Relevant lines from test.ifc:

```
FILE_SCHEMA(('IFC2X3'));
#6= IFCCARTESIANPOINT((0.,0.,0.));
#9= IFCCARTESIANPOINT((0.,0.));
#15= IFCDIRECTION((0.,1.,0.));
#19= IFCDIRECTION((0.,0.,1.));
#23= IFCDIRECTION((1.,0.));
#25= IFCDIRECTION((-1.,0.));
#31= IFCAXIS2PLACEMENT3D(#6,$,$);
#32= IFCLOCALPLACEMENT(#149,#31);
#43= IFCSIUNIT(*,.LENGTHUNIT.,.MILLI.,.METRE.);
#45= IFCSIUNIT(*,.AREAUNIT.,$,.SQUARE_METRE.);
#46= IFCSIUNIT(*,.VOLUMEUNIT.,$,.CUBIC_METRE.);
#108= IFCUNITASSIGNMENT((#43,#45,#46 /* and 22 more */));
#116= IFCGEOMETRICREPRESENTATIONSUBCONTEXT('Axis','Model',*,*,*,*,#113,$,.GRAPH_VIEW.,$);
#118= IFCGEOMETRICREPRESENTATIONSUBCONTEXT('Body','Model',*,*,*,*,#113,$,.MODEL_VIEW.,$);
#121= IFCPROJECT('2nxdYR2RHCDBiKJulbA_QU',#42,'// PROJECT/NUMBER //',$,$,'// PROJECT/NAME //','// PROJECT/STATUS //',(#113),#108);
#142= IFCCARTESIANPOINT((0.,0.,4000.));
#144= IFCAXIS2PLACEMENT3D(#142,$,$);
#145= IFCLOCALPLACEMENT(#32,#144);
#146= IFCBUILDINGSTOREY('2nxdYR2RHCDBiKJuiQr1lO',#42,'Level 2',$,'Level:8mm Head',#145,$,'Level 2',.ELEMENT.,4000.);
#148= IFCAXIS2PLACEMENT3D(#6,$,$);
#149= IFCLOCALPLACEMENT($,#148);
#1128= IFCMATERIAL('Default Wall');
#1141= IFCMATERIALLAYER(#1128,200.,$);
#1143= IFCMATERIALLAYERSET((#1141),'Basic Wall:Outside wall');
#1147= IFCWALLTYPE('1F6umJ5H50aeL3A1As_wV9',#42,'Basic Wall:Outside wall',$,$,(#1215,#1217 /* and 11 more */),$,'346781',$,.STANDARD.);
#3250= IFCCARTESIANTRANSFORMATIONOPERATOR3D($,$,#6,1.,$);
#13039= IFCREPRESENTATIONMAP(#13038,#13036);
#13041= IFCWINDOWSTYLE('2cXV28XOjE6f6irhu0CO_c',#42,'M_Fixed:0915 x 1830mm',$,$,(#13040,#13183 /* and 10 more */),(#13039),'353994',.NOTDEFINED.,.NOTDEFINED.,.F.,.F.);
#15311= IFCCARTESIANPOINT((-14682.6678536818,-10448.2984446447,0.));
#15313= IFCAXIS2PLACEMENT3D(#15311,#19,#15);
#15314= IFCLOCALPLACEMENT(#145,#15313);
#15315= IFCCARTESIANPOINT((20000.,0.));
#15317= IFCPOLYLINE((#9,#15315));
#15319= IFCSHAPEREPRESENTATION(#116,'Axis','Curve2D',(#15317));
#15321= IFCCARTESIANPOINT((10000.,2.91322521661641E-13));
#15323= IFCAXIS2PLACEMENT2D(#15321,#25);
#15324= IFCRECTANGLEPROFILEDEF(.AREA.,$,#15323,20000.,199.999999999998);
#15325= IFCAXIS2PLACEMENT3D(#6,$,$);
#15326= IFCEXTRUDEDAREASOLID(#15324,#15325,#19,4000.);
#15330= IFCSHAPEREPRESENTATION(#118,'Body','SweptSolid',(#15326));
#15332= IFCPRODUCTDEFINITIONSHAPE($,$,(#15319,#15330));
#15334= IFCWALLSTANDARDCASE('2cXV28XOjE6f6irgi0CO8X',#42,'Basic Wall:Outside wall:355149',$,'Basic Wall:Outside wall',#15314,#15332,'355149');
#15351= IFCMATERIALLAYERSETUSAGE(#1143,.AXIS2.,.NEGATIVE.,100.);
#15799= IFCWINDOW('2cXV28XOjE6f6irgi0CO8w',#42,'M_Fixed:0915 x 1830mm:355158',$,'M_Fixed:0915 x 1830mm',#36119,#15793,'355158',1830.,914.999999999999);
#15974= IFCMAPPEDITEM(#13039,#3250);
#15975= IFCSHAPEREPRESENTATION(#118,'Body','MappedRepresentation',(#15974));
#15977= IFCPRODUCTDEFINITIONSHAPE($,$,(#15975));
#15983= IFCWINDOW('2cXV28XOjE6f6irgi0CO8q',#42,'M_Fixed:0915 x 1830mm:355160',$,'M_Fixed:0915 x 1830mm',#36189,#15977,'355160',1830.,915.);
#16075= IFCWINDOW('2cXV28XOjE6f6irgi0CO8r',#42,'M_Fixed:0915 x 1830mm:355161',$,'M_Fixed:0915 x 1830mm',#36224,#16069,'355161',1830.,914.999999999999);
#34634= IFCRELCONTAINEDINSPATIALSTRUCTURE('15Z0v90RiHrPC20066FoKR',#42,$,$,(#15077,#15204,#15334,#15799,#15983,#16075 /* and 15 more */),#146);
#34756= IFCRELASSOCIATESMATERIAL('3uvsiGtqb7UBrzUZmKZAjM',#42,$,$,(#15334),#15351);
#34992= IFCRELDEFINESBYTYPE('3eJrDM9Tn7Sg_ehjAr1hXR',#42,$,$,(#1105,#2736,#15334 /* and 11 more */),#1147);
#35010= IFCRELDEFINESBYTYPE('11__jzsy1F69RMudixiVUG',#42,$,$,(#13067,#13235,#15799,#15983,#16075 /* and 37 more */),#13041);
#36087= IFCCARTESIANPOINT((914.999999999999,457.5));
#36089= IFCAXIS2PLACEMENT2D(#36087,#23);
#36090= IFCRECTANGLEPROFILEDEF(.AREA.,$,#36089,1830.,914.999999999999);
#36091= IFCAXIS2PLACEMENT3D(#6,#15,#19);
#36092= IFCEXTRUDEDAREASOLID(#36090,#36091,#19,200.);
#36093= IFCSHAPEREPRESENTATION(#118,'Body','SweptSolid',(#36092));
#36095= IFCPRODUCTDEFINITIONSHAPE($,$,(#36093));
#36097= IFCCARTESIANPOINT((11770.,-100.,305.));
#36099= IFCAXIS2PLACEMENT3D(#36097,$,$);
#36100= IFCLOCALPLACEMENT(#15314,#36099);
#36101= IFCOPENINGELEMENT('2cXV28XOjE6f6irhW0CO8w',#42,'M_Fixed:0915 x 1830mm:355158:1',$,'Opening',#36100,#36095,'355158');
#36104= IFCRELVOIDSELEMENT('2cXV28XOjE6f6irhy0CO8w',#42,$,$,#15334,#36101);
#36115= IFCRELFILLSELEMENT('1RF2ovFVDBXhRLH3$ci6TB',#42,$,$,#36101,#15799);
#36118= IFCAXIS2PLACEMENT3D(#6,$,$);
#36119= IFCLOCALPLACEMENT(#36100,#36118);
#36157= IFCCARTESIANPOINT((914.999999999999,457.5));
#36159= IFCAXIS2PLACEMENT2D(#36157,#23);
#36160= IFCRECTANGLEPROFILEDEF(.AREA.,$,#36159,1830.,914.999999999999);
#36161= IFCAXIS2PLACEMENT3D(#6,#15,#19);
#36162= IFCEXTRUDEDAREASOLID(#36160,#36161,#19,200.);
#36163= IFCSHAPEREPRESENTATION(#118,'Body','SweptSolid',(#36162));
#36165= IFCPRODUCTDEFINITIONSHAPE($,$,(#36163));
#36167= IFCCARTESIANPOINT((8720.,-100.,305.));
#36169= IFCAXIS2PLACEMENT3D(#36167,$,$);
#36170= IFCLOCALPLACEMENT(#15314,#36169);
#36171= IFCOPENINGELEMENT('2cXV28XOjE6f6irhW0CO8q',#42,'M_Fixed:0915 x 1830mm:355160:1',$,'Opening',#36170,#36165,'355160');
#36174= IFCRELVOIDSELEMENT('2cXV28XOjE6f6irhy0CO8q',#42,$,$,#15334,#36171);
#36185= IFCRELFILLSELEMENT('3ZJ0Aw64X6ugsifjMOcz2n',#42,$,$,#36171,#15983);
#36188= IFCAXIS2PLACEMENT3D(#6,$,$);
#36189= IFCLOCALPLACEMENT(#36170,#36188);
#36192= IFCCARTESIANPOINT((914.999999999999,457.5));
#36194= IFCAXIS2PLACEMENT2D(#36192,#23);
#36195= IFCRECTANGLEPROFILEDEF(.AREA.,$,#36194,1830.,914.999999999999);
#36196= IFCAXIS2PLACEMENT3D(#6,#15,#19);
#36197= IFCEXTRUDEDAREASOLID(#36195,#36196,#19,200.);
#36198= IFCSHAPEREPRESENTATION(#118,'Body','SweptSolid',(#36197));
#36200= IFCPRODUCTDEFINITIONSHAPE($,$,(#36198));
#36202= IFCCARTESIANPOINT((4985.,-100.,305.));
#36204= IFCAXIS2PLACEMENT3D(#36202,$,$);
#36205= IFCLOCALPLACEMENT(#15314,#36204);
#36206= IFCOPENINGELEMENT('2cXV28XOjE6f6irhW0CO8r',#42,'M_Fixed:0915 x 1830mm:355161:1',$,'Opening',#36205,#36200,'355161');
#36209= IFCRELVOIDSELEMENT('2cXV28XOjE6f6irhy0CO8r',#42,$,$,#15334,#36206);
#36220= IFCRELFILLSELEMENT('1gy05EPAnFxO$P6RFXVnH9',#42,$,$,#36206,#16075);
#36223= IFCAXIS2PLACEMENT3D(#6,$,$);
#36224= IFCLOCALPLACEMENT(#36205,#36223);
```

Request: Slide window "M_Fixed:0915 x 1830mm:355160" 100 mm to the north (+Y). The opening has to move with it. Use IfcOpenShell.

```python
import ifcopenshell
import ifcopenshell.api.geometry
import ifcopenshell.util.placement
import ifcopenshell.util.unit

model = ifcopenshell.open("test.ifc")
unit_scale = ifcopenshell.util.unit.calculate_unit_scale(model)

window = model.by_guid("2cXV28XOjE6f6irgi0CO8q")
opening = window.FillsVoids[0].RelatingOpeningElement
wall = opening.VoidsElements[0].RelatingBuildingElement

wall_matrix = ifcopenshell.util.placement.get_local_placement(wall.ObjectPlacement)
shift = wall_matrix[:3, 0] * 0.1 / unit_scale
before = ifcopenshell.util.placement.get_local_placement(window.ObjectPlacement)[:3, 3].copy()

# The window is placed relative to its opening, so it follows when the opening moves.
matrix = ifcopenshell.util.placement.get_local_placement(opening.ObjectPlacement)
matrix[:3, 3] += shift
ifcopenshell.api.geometry.edit_object_placement(
    model, product=opening, matrix=matrix, is_si=False, should_transform_children=True
)

after = ifcopenshell.util.placement.get_local_placement(window.ObjectPlacement)[:3, 3]
print("window moved by", (after - before).round(3) + 0.0)

model.write("test_rev.ifc")
```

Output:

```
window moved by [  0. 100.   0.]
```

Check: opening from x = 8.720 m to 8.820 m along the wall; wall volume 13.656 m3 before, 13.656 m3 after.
